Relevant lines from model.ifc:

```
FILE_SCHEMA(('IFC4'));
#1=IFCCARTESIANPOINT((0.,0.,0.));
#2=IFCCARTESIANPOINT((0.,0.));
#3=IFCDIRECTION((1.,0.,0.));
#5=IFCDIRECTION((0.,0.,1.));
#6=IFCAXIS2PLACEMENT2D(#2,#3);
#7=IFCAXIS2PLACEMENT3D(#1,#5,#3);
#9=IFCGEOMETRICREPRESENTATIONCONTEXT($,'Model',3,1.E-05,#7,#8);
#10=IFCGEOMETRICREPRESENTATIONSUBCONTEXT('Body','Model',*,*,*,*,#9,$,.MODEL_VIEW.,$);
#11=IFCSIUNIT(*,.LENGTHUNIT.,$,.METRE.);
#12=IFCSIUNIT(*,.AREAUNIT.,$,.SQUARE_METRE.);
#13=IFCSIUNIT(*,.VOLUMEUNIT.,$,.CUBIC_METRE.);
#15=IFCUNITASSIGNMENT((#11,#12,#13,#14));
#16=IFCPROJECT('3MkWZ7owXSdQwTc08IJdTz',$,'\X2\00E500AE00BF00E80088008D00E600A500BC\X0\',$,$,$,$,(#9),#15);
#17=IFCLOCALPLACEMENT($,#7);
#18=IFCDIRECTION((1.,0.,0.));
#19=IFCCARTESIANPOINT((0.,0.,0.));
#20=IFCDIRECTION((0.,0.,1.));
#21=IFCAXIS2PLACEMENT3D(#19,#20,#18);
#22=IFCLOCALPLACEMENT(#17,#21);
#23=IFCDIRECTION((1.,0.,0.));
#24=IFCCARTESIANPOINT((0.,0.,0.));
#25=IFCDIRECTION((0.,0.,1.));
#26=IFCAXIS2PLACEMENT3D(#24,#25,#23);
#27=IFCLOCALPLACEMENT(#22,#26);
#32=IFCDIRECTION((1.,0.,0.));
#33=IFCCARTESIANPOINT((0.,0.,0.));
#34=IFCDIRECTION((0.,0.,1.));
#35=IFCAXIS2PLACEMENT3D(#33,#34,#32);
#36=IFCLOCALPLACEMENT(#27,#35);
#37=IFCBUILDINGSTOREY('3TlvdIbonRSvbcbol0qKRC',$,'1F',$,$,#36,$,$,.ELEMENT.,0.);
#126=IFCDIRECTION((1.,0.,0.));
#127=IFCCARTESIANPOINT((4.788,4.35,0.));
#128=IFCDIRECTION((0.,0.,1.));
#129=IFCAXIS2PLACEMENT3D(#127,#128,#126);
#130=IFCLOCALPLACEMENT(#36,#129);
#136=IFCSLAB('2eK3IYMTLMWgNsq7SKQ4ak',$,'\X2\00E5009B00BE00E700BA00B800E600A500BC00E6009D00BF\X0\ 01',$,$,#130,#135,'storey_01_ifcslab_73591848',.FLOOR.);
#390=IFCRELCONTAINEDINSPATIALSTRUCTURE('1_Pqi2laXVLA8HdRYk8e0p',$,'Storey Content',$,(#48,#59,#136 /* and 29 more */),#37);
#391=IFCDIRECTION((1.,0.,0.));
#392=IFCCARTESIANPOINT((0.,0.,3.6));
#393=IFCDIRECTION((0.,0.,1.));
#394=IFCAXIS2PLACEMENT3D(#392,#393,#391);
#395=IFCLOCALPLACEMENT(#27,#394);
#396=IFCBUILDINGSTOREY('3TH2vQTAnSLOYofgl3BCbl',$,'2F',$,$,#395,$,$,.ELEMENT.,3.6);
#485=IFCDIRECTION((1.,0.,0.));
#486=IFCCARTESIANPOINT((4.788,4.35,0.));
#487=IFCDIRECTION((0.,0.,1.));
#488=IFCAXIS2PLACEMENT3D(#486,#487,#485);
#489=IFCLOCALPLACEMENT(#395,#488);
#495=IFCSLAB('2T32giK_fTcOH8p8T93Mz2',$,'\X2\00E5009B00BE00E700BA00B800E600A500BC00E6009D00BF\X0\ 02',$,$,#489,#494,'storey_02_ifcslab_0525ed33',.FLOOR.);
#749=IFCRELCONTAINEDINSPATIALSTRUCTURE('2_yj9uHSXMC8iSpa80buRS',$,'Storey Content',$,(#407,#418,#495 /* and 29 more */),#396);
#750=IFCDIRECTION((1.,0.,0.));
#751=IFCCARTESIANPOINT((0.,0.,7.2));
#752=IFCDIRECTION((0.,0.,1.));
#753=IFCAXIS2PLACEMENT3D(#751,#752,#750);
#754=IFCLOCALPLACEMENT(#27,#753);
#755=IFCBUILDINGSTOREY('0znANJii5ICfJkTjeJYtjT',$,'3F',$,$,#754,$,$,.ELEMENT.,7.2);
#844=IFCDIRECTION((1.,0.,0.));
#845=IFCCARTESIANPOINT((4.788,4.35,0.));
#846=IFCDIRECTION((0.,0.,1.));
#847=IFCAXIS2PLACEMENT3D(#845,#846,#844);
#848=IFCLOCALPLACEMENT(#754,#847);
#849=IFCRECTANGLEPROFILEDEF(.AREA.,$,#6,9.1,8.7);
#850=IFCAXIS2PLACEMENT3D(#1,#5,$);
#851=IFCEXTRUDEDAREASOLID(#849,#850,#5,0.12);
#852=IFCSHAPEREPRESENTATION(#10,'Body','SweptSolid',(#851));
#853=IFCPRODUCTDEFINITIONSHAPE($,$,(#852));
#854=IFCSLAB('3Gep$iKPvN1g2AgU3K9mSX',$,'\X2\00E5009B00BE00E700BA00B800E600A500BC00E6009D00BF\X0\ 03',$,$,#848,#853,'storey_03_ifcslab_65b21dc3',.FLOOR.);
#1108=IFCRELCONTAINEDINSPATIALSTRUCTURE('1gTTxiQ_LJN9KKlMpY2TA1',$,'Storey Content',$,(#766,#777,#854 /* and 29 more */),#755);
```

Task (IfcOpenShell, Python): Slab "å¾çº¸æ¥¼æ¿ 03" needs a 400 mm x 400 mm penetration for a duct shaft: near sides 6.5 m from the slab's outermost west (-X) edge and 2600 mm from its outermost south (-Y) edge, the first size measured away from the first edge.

```python
import numpy as np
import ifcopenshell
import ifcopenshell.api.feature
import ifcopenshell.api.geometry
import ifcopenshell.api.root
import ifcopenshell.geom
import ifcopenshell.util.placement
import ifcopenshell.util.representation
import ifcopenshell.util.shape
import ifcopenshell.util.unit

model = ifcopenshell.open("model.ifc")
unit_scale = ifcopenshell.util.unit.calculate_unit_scale(model)
settings = ifcopenshell.geom.settings()


def volume(element):
    """Net volume in cubic metres, openings subtracted."""
    shape = ifcopenshell.geom.create_shape(settings, element)
    return ifcopenshell.util.shape.get_volume(shape.geometry)


slab = model.by_guid("3Gep$iKPvN1g2AgU3K9mSX")
before = volume(slab)

# Extent in the slab's own axes, in metres. The edges named are its -X and -Y sides.
slab_shape = ifcopenshell.geom.create_shape(settings, slab)
vertices = ifcopenshell.util.shape.get_vertices(slab_shape.geometry)
x_min, y_min, bottom = vertices.min(axis=0)
top = vertices[:, 2].max()

opening = ifcopenshell.api.root.create_entity(model, ifc_class="IfcOpeningElement", name="Duct shaft opening", predefined_type="OPENING")
context = ifcopenshell.util.representation.get_context(model, "Model", "Body", "MODEL_VIEW")
width, depth = 0.4, 0.4
outline = [(0.0, 0.0), (width, 0.0), (width, depth), (0.0, depth), (0.0, 0.0)]
# Overshoot both faces by 50 mm so the cut is clean.
shape = ifcopenshell.api.geometry.add_slab_representation(
    model, context=context, depth=top - bottom + 0.1, polyline=outline
)
ifcopenshell.api.geometry.assign_representation(model, product=opening, representation=shape)

matrix = ifcopenshell.util.placement.get_local_placement(slab.ObjectPlacement)
matrix[:, 3] = matrix @ np.append(np.array([x_min + 6.5, y_min + 2.6, bottom - 0.05]) / unit_scale, 1.0)
ifcopenshell.api.geometry.edit_object_placement(model, product=opening, matrix=matrix, is_si=False)
ifcopenshell.api.feature.add_feature(model, feature=opening, element=slab)

after = volume(slab)

print(f"slab volume {before:.3f} -> {after:.3f} m3")

model.write("model_v2.ifc")
```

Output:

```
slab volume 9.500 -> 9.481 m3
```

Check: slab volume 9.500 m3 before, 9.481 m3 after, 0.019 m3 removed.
